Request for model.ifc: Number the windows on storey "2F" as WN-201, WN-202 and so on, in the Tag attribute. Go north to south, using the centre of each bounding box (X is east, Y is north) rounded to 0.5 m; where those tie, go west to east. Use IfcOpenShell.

First a look at what the model holds.

```python
import ifcopenshell
import ifcopenshell.util.element
import ifcopenshell.util.placement

model = ifcopenshell.open("model.ifc")
print(model.schema)
storey = next(s for s in model.by_type("IfcBuildingStorey") if s.Name == "2F")
windows = [e for e in ifcopenshell.util.element.get_decomposition(storey) if e.is_a("IfcWindow")]
for e in sorted(windows, key=lambda e: e.id()):
    origin = ifcopenshell.util.placement.get_local_placement(e.ObjectPlacement)[:3, 3]
    print(e.id(), e.Tag, e.Name, origin.round(2) + 0.0, sep=" | ")
```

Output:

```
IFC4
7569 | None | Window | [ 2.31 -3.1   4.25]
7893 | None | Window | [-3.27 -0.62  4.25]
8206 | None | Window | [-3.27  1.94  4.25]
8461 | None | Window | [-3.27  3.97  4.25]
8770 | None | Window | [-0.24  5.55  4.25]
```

```python
import ifcopenshell
import ifcopenshell.geom
import ifcopenshell.util.element
import ifcopenshell.util.shape

model = ifcopenshell.open("model.ifc")
settings = ifcopenshell.geom.settings()
settings.set("use-world-coords", True)


def centre(element):
    shape = ifcopenshell.geom.create_shape(settings, element)
    return ifcopenshell.util.shape.get_bbox_centroid(shape.geometry)


storey = next(s for s in model.by_type("IfcBuildingStorey") if s.Name == "2F")
windows = [e for e in ifcopenshell.util.element.get_decomposition(storey) if e.is_a("IfcWindow")]

# Insertion points can sit at a corner or the storey origin, so sort by the geometry (in metres).
centres = {e: centre(e) for e in windows}
windows.sort(key=lambda e: (-round(centres[e][1] / 0.5), centres[e][0]))

for i, e in enumerate(windows, start=1):
    number = f"WN-2{i:02d}"
    e.Tag = number
    print(e.id(), number)

model.write("model_edited.ifc")
```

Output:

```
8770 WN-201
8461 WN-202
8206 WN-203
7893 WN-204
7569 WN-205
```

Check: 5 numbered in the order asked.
